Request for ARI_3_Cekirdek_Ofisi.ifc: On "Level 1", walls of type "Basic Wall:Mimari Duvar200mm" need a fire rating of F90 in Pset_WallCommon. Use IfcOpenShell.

First a look at what the model holds.

```python
import ifcopenshell
import ifcopenshell.util.element

model = ifcopenshell.open("ARI_3_Cekirdek_Ofisi.ifc")
print(model.schema)
storey = next(s for s in model.by_type("IfcBuildingStorey") if s.Name == "Level 1")
walls = [e for e in ifcopenshell.util.element.get_decomposition(storey) if e.is_a("IfcWall")]
seen = {}
for e in walls:
    element_type = ifcopenshell.util.element.get_type(e)
    key = (element_type.Name if element_type != e and element_type else None, ifcopenshell.util.element.get_pset(e, "Pset_WallCommon", "FireRating"))
    seen[key] = seen.get(key, 0) + 1
for (name, value), count in sorted(seen.items(), key=str):
    print(count, "x", name, "|", value)
```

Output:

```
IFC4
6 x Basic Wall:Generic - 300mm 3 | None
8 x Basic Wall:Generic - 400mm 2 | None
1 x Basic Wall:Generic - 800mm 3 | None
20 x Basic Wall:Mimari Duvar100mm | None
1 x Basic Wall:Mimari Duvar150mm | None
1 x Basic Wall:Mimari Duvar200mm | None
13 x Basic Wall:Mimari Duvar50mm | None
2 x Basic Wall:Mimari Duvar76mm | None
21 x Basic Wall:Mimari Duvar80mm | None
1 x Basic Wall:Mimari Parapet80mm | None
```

```python
import ifcopenshell
import ifcopenshell.api.pset
import ifcopenshell.util.element

model = ifcopenshell.open("ARI_3_Cekirdek_Ofisi.ifc")

storey = next(s for s in model.by_type("IfcBuildingStorey") if s.Name == "Level 1")
walls = [e for e in ifcopenshell.util.element.get_decomposition(storey) if e.is_a("IfcWall")]

count = 0
for e in walls:
    element_type = ifcopenshell.util.element.get_type(e)
    if element_type in (None, e) or element_type.Name != "Basic Wall:Mimari Duvar200mm":
        continue
    # add_pset returns the element's existing set when there is one.
    pset = ifcopenshell.api.pset.add_pset(model, product=e, name="Pset_WallCommon")
    ifcopenshell.api.pset.edit_pset(model, pset=pset, properties={"FireRating": "F90"})
    count += 1

print(count, "walls updated")

model.write("ARI_3_Cekirdek_Ofisi_rev.ifc")
```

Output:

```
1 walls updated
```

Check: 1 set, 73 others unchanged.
